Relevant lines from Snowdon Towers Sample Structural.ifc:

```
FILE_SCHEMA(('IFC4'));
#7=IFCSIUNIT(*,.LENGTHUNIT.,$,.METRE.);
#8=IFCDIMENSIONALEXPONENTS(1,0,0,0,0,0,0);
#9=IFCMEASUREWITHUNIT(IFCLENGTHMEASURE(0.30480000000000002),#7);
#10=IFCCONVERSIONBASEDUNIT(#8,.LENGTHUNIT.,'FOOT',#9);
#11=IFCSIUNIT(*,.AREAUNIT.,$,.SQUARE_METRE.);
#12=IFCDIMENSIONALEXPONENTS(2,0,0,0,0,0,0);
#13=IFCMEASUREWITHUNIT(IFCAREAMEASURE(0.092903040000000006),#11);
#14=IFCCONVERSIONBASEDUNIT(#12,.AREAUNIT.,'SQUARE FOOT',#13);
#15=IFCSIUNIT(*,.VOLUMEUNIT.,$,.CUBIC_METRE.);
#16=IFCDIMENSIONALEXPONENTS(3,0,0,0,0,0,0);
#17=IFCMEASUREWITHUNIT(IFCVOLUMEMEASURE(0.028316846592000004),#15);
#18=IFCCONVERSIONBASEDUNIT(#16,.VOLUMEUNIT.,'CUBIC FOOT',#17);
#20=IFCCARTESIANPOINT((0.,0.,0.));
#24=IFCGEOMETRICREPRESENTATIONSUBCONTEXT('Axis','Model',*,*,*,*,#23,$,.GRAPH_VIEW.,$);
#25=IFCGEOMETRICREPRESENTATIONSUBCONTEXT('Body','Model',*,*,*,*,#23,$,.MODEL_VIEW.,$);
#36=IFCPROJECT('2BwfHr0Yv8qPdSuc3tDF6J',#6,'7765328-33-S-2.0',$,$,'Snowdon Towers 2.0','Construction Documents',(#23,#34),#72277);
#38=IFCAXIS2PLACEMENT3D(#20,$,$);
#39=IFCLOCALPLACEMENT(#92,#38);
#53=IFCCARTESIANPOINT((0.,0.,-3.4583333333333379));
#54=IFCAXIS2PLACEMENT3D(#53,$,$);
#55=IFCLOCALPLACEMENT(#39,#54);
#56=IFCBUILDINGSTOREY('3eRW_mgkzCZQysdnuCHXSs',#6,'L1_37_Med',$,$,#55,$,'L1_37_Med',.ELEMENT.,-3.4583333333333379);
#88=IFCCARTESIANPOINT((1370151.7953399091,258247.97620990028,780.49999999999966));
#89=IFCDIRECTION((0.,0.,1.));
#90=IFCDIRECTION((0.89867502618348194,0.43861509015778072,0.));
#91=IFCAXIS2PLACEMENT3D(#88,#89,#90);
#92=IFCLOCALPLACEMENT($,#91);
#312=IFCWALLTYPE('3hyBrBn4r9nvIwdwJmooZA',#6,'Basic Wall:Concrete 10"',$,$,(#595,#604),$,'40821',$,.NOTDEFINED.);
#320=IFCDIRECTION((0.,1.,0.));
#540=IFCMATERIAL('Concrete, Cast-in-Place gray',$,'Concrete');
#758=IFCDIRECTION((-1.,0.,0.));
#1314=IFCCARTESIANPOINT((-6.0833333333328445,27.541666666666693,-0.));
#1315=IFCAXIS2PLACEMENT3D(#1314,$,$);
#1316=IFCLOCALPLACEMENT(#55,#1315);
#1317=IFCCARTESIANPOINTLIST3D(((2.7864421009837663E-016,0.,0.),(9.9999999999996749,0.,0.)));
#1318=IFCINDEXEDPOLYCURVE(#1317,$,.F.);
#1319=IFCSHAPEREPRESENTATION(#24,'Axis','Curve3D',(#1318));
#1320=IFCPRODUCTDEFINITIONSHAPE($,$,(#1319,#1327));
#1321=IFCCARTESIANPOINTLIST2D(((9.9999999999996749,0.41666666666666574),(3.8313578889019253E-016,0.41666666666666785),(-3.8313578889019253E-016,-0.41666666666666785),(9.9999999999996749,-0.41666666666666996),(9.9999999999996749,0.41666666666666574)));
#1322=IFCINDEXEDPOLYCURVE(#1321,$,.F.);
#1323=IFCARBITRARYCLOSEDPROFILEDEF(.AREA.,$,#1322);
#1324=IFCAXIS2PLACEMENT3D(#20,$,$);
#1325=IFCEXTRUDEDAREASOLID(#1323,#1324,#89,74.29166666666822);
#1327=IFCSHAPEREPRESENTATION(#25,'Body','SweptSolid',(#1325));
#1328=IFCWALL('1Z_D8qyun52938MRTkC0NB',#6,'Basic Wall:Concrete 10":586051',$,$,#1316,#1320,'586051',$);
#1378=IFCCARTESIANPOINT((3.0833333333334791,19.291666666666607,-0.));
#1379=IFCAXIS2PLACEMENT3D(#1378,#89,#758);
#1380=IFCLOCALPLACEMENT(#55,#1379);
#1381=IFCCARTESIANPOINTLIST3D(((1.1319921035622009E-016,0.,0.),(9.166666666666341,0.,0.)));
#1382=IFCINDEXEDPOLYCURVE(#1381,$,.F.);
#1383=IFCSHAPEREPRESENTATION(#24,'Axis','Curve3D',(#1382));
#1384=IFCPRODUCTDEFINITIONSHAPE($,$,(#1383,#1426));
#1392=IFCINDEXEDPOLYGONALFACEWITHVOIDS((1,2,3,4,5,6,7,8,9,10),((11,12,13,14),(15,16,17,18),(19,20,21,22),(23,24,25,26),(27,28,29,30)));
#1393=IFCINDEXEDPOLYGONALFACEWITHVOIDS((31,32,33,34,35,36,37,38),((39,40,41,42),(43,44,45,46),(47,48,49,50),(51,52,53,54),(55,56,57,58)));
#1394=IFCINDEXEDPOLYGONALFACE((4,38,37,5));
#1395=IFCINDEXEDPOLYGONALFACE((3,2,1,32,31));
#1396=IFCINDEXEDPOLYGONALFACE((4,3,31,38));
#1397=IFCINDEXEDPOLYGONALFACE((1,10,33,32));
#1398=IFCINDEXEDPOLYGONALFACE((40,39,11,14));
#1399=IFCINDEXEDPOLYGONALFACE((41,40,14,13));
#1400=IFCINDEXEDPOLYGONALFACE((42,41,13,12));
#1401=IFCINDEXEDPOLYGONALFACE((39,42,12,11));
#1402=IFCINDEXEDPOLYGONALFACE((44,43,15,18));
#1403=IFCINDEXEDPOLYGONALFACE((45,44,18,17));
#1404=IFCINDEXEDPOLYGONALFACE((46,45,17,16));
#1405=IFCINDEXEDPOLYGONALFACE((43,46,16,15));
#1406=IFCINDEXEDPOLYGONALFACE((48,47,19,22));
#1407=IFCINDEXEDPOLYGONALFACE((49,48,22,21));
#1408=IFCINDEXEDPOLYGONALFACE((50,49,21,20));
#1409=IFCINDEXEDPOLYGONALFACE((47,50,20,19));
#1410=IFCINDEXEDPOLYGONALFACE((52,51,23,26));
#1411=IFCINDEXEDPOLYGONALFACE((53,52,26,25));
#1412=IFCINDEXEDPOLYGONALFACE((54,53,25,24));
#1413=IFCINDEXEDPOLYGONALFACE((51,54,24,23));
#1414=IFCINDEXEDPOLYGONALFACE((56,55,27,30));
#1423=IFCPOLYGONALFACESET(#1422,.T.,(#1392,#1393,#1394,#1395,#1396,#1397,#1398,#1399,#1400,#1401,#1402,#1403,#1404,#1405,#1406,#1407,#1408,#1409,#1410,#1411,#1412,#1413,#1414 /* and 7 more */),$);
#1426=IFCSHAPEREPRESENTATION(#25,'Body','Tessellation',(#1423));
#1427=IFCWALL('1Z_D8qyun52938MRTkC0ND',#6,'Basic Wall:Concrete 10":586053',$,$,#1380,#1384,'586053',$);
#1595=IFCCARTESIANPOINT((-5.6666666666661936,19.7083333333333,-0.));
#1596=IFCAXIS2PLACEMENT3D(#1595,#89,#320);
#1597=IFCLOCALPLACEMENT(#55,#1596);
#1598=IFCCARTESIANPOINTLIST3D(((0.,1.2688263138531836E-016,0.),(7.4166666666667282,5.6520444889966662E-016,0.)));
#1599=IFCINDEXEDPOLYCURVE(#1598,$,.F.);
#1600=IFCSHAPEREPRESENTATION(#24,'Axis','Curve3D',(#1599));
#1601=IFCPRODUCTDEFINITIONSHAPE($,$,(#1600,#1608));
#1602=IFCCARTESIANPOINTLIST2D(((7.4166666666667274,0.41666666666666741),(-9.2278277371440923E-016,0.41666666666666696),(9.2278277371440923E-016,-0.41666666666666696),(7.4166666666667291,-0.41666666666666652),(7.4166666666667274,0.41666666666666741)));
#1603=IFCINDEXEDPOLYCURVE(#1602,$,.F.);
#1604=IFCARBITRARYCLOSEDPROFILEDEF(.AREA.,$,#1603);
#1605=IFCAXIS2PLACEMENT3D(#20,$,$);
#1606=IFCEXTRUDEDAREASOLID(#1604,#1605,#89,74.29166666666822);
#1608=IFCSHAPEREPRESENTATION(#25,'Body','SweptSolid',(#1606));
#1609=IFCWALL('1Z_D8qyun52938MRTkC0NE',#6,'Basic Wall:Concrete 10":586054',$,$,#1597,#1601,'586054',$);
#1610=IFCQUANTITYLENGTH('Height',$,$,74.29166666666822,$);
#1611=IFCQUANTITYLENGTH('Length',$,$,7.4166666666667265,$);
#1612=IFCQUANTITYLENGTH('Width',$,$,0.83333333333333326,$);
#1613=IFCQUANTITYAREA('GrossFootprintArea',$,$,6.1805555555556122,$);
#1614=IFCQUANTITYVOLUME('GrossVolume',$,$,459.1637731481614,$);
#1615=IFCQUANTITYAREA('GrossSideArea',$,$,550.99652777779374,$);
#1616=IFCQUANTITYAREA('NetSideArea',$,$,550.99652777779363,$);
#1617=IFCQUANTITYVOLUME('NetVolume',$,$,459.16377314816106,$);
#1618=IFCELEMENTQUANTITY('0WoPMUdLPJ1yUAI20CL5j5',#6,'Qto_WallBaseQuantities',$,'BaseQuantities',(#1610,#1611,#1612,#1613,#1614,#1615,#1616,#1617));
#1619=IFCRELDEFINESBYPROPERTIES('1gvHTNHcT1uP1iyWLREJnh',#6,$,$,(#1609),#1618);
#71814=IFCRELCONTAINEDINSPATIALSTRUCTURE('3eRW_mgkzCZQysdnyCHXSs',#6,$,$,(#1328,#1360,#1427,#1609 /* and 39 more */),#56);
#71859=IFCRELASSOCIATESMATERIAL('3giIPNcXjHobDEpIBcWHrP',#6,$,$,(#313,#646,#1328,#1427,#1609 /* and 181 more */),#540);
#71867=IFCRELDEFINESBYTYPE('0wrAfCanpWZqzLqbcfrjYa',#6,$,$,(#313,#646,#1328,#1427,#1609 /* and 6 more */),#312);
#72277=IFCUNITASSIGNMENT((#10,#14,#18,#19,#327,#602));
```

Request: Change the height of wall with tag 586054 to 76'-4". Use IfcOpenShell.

```python
import ifcopenshell
import ifcopenshell.api.pset
import ifcopenshell.geom
import ifcopenshell.util.element
import ifcopenshell.util.representation
import ifcopenshell.util.shape
import ifcopenshell.util.unit

model = ifcopenshell.open("Snowdon Towers Sample Structural.ifc")
unit_scale = ifcopenshell.util.unit.calculate_unit_scale(model)
area_scale = ifcopenshell.util.unit.calculate_unit_scale(model, "AREAUNIT")
volume_scale = ifcopenshell.util.unit.calculate_unit_scale(model, "VOLUMEUNIT")
settings = ifcopenshell.geom.settings()


def volume(element):
    """Net volume in cubic metres, openings subtracted."""
    shape = ifcopenshell.geom.create_shape(settings, element)
    return ifcopenshell.util.shape.get_volume(shape.geometry)


wall = model.by_id(1609)
before = volume(wall)

body = ifcopenshell.util.representation.get_representation(wall, "Model", "Body")
solid = body.Items[0]
old_height = solid.Depth
solid.Depth = 916 * 0.0254 / unit_scale
after = volume(wall)
thickness = 0.254  # wall thickness in metres

# Update the stored height, areas and volumes.
qto = model.by_id(ifcopenshell.util.element.get_pset(wall, "Qto_WallBaseQuantities", should_inherit=False)["id"])
ifcopenshell.api.pset.edit_qto(model, qto=qto, properties={
    "Height": solid.Depth,
    "GrossVolume": ifcopenshell.util.element.get_pset(wall, "Qto_WallBaseQuantities", "GrossVolume") * solid.Depth / old_height,
    "GrossSideArea": ifcopenshell.util.element.get_pset(wall, "Qto_WallBaseQuantities", "GrossSideArea") * solid.Depth / old_height,
    "NetSideArea": after / thickness / area_scale,
    "NetVolume": after / volume_scale,
})

print(f"height {old_height:g} -> {solid.Depth:g}, volume {before:.3f} -> {after:.3f} m3")

model.write("Snowdon Towers Sample Structural_v2.ifc")
```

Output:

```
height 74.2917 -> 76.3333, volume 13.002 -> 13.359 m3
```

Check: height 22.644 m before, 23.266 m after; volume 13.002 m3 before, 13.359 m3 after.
